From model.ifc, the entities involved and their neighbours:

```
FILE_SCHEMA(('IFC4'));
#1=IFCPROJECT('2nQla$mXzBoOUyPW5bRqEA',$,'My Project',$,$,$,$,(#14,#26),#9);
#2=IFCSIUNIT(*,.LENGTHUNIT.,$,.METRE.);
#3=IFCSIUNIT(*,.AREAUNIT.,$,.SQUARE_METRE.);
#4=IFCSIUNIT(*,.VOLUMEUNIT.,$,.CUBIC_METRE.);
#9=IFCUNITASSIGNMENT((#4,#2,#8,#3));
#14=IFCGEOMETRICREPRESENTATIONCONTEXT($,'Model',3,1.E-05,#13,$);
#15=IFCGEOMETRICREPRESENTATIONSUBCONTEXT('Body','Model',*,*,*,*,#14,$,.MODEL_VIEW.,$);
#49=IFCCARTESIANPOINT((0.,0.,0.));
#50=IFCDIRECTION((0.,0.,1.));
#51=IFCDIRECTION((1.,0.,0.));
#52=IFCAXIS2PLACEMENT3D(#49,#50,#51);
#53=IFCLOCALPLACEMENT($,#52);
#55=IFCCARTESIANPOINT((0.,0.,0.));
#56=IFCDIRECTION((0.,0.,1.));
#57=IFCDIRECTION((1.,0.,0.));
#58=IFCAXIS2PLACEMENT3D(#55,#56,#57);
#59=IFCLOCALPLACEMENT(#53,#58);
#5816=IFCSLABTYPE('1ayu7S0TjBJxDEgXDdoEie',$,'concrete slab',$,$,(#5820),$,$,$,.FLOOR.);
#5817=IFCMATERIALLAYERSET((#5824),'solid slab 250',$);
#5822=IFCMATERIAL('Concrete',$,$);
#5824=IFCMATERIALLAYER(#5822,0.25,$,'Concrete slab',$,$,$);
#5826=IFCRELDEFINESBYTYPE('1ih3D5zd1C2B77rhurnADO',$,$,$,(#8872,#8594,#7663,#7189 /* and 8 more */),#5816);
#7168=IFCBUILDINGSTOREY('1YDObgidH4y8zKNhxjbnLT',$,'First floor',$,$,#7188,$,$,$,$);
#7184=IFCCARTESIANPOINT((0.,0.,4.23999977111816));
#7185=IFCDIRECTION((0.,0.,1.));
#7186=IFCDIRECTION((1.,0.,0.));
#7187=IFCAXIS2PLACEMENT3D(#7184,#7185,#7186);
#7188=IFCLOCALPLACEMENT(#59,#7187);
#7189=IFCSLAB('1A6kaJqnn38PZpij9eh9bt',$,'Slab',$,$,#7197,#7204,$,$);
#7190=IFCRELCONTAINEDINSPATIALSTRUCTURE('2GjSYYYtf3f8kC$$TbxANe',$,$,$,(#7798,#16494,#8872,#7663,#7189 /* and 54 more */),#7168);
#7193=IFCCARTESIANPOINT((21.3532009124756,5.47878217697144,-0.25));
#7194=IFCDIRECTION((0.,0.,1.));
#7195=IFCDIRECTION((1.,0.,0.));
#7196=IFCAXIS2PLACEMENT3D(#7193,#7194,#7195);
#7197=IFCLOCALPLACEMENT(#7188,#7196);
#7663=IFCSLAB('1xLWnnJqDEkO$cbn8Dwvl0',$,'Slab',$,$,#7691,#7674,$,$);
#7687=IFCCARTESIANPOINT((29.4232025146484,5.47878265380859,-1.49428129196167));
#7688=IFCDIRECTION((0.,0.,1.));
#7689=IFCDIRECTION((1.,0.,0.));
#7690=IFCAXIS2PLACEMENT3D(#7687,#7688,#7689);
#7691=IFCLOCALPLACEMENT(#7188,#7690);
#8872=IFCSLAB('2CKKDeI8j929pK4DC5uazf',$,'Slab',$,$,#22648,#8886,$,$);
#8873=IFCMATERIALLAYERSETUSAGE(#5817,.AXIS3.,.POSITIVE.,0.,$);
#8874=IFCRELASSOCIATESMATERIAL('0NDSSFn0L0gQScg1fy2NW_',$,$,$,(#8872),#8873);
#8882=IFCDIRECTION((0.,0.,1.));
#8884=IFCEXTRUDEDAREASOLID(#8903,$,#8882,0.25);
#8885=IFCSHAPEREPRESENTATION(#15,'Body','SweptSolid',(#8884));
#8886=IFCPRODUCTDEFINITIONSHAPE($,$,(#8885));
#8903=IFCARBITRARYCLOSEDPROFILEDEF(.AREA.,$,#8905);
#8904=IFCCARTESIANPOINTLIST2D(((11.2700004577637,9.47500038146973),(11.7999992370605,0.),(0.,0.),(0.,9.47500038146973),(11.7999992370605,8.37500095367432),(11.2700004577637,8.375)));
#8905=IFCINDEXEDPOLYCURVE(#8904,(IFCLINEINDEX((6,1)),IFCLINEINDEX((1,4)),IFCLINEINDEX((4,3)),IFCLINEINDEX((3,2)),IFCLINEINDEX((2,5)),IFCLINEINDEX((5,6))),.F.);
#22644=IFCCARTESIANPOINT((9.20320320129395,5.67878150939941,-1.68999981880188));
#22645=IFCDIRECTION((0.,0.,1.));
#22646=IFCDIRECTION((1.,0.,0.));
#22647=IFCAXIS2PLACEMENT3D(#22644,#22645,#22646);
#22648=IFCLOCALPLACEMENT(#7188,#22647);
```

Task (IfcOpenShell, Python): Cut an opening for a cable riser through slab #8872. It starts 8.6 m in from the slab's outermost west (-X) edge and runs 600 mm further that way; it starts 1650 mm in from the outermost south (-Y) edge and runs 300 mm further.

```python
import numpy as np
import ifcopenshell
import ifcopenshell.api.feature
import ifcopenshell.api.geometry
import ifcopenshell.api.root
import ifcopenshell.geom
import ifcopenshell.util.placement
import ifcopenshell.util.representation
import ifcopenshell.util.shape
import ifcopenshell.util.unit

model = ifcopenshell.open("model.ifc")
unit_scale = ifcopenshell.util.unit.calculate_unit_scale(model)
settings = ifcopenshell.geom.settings()


def volume(element):
    """Net volume in cubic metres, openings subtracted."""
    shape = ifcopenshell.geom.create_shape(settings, element)
    return ifcopenshell.util.shape.get_volume(shape.geometry)


slab = model.by_guid("2CKKDeI8j929pK4DC5uazf")
before = volume(slab)

# Extent in the slab's own axes, in metres. The edges named are its -X and -Y sides.
slab_shape = ifcopenshell.geom.create_shape(settings, slab)
vertices = ifcopenshell.util.shape.get_vertices(slab_shape.geometry)
x_min, y_min, bottom = vertices.min(axis=0)
top = vertices[:, 2].max()

opening = ifcopenshell.api.root.create_entity(model, ifc_class="IfcOpeningElement", name="Cable riser opening", predefined_type="OPENING")
context = ifcopenshell.util.representation.get_context(model, "Model", "Body", "MODEL_VIEW")
width, depth = 0.6, 0.3
outline = [(0.0, 0.0), (width, 0.0), (width, depth), (0.0, depth), (0.0, 0.0)]
# Overshoot both faces by 50 mm so the cut is clean.
shape = ifcopenshell.api.geometry.add_slab_representation(
    model, context=context, depth=top - bottom + 0.1, polyline=outline
)
ifcopenshell.api.geometry.assign_representation(model, product=opening, representation=shape)

matrix = ifcopenshell.util.placement.get_local_placement(slab.ObjectPlacement)
matrix[:, 3] = matrix @ np.append(np.array([x_min + 8.6, y_min + 1.65, bottom - 0.05]) / unit_scale, 1.0)
ifcopenshell.api.geometry.edit_object_placement(model, product=opening, matrix=matrix, is_si=False)
ifcopenshell.api.feature.add_feature(model, feature=opening, element=slab)

after = volume(slab)

print(f"slab volume {before:.3f} -> {after:.3f} m3")

model.write("model_rev.ifc")
```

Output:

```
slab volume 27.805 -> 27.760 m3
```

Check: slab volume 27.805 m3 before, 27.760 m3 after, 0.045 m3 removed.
